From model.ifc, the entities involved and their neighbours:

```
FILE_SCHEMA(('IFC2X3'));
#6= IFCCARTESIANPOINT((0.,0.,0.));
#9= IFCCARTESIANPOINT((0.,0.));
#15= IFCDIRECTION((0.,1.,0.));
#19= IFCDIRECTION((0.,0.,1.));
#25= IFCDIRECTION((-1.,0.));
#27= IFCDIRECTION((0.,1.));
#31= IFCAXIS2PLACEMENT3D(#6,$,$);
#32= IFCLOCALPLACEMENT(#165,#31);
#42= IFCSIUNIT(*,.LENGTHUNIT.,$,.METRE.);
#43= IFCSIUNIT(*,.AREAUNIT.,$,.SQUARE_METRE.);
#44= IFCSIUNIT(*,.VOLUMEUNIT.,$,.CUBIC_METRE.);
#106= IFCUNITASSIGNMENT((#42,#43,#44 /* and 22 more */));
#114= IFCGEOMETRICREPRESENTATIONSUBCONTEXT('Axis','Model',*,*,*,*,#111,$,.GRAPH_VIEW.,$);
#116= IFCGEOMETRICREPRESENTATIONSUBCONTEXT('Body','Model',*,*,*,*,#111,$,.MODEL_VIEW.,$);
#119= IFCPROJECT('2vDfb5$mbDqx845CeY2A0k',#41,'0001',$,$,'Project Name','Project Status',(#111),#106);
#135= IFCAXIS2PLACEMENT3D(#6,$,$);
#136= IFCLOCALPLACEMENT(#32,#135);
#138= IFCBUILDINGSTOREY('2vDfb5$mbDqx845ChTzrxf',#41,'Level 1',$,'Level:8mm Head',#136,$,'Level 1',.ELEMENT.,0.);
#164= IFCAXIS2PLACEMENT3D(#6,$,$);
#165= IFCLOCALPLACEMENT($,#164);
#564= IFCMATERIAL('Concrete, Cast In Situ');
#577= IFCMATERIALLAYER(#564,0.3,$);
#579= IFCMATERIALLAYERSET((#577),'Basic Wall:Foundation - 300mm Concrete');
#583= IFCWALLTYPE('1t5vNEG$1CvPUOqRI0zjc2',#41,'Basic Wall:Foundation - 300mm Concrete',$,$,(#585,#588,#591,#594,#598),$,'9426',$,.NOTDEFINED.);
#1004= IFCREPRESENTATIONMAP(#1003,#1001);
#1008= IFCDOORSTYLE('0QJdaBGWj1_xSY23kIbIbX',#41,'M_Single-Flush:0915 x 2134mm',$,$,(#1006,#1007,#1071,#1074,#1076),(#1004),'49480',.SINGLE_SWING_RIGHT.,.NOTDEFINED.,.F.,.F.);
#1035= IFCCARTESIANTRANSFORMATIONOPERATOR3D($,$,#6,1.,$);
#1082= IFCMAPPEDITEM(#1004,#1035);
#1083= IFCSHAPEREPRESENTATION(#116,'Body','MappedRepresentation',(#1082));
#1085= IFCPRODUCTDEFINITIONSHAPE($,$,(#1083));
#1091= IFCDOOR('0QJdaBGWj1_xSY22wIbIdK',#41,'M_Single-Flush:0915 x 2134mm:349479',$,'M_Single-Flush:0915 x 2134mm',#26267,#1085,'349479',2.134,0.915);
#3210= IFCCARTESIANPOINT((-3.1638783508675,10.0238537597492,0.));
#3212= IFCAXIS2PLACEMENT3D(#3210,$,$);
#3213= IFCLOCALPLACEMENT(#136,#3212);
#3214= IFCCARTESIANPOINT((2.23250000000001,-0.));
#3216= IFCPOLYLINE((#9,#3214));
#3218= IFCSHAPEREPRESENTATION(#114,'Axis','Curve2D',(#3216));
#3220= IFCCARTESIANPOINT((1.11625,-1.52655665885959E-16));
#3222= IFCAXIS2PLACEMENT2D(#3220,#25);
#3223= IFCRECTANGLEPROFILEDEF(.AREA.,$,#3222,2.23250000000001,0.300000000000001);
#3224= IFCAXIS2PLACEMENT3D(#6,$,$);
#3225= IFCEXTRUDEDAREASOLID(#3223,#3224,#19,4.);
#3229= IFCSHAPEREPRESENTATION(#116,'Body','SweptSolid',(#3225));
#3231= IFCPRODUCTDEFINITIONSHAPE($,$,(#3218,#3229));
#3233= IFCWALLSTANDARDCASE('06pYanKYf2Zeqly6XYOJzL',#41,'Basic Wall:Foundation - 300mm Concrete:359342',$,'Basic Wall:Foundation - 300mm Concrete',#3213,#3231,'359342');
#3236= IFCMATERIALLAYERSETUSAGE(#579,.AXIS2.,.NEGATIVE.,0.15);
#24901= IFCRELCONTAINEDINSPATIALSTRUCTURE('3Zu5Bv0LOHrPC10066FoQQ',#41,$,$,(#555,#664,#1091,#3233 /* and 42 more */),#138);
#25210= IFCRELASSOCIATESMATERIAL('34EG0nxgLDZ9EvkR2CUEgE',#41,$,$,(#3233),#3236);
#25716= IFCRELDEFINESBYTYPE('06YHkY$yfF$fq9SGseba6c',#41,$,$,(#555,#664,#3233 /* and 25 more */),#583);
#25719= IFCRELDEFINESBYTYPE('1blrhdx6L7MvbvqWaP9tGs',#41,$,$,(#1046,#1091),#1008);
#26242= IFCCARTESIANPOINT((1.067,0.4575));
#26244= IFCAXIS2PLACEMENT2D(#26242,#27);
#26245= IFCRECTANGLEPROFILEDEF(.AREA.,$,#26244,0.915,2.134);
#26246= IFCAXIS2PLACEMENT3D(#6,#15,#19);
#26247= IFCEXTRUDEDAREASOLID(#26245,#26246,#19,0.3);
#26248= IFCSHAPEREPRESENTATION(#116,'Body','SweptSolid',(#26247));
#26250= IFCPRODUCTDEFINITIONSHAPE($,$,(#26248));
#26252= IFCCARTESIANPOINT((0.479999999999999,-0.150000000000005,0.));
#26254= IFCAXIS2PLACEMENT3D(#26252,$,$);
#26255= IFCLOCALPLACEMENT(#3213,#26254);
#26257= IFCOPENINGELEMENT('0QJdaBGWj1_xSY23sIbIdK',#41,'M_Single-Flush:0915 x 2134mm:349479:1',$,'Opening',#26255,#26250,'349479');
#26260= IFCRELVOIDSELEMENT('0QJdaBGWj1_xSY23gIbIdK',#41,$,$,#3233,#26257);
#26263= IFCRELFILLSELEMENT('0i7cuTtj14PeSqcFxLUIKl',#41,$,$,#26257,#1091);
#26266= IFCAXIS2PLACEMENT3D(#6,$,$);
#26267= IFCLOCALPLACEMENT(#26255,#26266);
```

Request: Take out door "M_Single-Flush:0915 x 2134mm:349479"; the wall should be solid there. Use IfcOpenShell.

```python
import ifcopenshell
import ifcopenshell.api.feature
import ifcopenshell.api.root
import ifcopenshell.geom
import ifcopenshell.util.shape

model = ifcopenshell.open("model.ifc")
settings = ifcopenshell.geom.settings()


def volume(element):
    """Net volume in cubic metres, openings subtracted."""
    shape = ifcopenshell.geom.create_shape(settings, element)
    return ifcopenshell.util.shape.get_volume(shape.geometry)


door = model.by_guid("0QJdaBGWj1_xSY22wIbIdK")
opening = door.FillsVoids[0].RelatingOpeningElement
wall = opening.VoidsElements[0].RelatingBuildingElement
before = volume(wall)

ifcopenshell.api.root.remove_product(model, product=door)
ifcopenshell.api.feature.remove_feature(model, feature=opening)

after = volume(wall)

print(f"wall volume {before:.3f} -> {after:.3f} m3")

model.write("model_edited.ifc")
```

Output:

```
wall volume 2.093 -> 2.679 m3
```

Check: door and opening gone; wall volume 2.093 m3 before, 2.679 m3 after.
